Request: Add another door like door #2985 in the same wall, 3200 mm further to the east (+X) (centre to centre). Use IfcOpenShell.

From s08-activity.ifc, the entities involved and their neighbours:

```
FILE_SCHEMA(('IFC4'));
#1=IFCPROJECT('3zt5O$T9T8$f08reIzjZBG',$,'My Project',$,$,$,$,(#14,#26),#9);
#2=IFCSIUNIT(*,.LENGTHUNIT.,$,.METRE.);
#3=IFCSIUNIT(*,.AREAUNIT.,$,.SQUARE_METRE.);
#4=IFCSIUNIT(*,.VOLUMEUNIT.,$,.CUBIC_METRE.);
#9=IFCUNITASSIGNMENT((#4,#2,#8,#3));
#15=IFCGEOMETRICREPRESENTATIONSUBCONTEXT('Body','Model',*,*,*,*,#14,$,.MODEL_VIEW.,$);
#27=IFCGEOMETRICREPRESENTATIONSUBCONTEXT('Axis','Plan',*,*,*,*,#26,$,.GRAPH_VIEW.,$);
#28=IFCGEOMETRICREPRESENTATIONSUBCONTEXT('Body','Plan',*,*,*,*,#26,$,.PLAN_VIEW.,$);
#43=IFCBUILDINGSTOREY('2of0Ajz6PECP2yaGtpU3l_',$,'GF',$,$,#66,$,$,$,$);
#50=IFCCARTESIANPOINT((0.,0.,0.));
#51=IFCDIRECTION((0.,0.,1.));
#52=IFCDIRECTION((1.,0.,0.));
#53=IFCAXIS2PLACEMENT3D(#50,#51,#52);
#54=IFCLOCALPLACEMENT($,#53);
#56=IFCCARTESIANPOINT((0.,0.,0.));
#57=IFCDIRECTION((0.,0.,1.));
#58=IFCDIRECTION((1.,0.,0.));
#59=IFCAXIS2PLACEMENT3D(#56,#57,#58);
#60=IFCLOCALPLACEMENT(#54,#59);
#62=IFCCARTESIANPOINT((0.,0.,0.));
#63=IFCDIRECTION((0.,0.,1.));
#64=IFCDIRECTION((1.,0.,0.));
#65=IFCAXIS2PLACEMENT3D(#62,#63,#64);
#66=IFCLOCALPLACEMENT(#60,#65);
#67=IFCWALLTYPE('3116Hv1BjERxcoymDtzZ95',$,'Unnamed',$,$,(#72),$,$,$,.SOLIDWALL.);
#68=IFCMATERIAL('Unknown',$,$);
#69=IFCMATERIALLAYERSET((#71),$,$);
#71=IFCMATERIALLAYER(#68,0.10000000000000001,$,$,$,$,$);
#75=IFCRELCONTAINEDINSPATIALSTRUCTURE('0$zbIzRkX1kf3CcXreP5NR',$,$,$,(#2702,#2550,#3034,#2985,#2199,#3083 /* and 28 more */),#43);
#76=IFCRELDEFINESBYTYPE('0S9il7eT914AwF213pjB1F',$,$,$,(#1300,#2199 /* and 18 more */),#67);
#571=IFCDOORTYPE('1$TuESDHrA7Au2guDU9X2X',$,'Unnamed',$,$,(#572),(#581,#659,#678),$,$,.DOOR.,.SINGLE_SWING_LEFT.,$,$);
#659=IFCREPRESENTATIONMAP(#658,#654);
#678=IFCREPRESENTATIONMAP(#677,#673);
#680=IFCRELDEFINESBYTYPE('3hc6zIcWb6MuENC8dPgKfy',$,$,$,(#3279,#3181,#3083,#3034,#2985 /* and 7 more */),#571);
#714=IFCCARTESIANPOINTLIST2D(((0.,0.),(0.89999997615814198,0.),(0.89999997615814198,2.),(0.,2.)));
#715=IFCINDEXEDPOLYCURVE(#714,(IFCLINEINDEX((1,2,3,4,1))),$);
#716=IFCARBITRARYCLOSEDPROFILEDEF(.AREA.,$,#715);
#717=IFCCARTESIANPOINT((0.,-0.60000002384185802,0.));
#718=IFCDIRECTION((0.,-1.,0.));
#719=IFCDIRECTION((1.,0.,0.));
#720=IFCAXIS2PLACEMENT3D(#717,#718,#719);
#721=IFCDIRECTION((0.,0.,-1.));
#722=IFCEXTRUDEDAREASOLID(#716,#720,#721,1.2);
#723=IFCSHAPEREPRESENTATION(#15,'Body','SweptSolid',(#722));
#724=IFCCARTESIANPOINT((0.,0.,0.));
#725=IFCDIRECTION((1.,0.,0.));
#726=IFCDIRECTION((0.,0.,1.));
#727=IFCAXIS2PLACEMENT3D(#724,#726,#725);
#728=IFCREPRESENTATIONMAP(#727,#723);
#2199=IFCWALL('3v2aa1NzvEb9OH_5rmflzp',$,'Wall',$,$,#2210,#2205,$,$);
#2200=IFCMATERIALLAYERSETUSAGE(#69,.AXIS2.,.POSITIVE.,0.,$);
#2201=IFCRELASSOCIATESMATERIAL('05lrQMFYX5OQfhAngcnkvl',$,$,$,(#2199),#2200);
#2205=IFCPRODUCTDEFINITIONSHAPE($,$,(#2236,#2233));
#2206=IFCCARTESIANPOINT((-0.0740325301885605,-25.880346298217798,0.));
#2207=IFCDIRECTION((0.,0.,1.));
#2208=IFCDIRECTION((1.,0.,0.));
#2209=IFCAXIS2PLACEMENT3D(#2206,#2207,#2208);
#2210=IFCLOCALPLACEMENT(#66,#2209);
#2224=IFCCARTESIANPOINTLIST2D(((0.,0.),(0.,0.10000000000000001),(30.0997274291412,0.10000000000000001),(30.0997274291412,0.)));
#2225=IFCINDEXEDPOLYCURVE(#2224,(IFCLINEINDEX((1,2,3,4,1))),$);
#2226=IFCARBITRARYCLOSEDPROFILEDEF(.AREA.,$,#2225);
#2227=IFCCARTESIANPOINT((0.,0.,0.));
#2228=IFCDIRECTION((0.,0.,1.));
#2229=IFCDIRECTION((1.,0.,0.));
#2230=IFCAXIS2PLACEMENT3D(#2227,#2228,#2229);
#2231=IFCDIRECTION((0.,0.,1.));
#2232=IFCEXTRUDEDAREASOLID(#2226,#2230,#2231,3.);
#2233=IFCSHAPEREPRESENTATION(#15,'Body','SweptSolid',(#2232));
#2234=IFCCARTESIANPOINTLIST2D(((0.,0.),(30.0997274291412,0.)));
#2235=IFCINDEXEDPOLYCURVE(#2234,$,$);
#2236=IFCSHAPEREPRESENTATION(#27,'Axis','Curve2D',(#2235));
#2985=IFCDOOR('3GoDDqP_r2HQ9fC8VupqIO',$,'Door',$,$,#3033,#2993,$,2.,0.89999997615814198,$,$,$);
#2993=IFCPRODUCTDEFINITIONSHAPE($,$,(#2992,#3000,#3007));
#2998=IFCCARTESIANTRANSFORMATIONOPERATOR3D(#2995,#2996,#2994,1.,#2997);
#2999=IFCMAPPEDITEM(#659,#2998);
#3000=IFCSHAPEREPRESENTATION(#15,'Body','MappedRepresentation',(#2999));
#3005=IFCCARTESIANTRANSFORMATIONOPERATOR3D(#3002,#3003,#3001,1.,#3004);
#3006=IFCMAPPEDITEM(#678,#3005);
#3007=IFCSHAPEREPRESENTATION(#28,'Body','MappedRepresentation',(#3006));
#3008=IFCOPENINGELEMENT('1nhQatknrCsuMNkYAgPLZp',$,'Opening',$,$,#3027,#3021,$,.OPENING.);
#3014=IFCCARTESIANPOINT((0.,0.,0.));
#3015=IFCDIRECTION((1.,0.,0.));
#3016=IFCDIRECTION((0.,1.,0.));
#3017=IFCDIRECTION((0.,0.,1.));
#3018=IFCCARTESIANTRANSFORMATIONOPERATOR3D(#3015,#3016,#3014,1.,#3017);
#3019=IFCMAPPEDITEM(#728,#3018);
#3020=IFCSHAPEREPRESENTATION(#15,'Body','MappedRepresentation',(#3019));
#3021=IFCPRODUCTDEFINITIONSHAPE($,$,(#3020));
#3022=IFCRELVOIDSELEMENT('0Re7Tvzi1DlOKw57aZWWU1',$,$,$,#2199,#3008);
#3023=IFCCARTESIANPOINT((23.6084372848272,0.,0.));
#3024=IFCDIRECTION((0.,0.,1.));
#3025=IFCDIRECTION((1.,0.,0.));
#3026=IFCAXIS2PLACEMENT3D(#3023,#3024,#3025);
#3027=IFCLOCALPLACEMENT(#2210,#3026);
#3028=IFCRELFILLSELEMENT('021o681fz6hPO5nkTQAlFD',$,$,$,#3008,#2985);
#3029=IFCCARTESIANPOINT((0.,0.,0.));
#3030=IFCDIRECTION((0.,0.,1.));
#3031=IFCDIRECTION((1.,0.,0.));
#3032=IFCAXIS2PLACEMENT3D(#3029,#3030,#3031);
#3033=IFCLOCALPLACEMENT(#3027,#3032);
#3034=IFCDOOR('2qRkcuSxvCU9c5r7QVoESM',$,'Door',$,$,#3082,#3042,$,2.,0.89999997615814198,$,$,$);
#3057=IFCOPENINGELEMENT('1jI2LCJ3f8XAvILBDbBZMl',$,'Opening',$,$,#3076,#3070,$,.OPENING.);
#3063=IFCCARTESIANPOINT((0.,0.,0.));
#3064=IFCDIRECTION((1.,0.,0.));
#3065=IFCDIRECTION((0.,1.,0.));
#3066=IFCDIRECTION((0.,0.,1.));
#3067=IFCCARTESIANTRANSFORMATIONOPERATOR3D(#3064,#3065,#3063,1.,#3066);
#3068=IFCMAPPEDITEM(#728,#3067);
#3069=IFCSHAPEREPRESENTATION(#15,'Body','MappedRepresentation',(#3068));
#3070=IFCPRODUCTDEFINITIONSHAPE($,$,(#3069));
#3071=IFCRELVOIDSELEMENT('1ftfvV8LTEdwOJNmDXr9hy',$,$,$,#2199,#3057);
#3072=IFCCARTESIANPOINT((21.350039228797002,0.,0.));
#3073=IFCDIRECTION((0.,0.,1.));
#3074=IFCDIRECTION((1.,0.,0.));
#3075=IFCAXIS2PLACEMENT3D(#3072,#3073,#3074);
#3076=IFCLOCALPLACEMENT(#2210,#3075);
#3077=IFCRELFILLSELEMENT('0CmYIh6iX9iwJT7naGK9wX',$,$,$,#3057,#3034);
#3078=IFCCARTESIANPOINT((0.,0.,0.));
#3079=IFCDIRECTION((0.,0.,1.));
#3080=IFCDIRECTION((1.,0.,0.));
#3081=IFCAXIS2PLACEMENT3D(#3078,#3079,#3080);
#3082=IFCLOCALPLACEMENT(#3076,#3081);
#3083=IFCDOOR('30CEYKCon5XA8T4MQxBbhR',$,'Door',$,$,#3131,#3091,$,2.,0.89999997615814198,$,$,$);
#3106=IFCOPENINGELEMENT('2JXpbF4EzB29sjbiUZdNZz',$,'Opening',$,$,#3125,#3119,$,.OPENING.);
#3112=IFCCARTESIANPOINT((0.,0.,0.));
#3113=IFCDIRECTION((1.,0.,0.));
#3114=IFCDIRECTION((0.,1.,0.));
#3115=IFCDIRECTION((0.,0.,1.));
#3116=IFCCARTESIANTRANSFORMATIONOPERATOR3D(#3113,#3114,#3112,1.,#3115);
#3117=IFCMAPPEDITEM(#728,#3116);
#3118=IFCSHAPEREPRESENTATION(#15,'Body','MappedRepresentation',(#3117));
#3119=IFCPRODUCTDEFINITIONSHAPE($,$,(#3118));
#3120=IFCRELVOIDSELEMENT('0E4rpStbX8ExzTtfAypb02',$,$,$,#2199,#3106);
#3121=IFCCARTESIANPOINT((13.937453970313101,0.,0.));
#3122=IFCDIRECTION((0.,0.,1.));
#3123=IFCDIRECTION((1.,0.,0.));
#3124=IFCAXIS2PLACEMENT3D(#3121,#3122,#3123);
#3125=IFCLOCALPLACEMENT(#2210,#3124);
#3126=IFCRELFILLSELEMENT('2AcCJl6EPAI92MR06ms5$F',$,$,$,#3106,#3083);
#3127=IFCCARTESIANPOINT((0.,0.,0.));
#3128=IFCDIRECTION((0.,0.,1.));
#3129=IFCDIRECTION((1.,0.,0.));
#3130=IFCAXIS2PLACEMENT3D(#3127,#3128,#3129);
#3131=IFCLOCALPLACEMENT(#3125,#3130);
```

```python
import ifcopenshell
import ifcopenshell.api.feature
import ifcopenshell.api.geometry
import ifcopenshell.api.root
import ifcopenshell.geom
import ifcopenshell.util.element
import ifcopenshell.util.placement
import ifcopenshell.util.shape
import ifcopenshell.util.unit

model = ifcopenshell.open("s08-activity.ifc")
unit_scale = ifcopenshell.util.unit.calculate_unit_scale(model)
settings = ifcopenshell.geom.settings()


def volume(element):
    """Net volume in cubic metres, openings subtracted."""
    shape = ifcopenshell.geom.create_shape(settings, element)
    return ifcopenshell.util.shape.get_volume(shape.geometry)


door = model.by_guid("3GoDDqP_r2HQ9fC8VupqIO")
opening = door.FillsVoids[0].RelatingOpeningElement
wall = opening.VoidsElements[0].RelatingBuildingElement
before = volume(wall)
shift = ifcopenshell.util.placement.get_local_placement(wall.ObjectPlacement)[:3, 0] * 3.2 / unit_scale

# copy_class copies the void relationship, type, container and properties, but no geometry.
new_opening = ifcopenshell.api.root.copy_class(model, product=opening)
new_opening.Representation = ifcopenshell.util.element.copy_deep(
    model, opening.Representation, exclude=["IfcGeometricRepresentationContext", "IfcRepresentationMap"]
)
new_door = ifcopenshell.api.root.copy_class(model, product=door)
new_door.Representation = ifcopenshell.util.element.copy_deep(
    model, door.Representation, exclude=["IfcGeometricRepresentationContext", "IfcRepresentationMap"]
)
ifcopenshell.api.feature.add_filling(model, opening=new_opening, element=new_door)

for old, new in ((opening, new_opening), (door, new_door)):
    matrix = ifcopenshell.util.placement.get_local_placement(old.ObjectPlacement)
    matrix[:3, 3] += shift
    ifcopenshell.api.geometry.edit_object_placement(model, product=new, matrix=matrix, is_si=False)

after = volume(wall)

print(f"wall volume {before:.3f} -> {after:.3f} m3")

model.write("s08-activity_updated.ifc")
```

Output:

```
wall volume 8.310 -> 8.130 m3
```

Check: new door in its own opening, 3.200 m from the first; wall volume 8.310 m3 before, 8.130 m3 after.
